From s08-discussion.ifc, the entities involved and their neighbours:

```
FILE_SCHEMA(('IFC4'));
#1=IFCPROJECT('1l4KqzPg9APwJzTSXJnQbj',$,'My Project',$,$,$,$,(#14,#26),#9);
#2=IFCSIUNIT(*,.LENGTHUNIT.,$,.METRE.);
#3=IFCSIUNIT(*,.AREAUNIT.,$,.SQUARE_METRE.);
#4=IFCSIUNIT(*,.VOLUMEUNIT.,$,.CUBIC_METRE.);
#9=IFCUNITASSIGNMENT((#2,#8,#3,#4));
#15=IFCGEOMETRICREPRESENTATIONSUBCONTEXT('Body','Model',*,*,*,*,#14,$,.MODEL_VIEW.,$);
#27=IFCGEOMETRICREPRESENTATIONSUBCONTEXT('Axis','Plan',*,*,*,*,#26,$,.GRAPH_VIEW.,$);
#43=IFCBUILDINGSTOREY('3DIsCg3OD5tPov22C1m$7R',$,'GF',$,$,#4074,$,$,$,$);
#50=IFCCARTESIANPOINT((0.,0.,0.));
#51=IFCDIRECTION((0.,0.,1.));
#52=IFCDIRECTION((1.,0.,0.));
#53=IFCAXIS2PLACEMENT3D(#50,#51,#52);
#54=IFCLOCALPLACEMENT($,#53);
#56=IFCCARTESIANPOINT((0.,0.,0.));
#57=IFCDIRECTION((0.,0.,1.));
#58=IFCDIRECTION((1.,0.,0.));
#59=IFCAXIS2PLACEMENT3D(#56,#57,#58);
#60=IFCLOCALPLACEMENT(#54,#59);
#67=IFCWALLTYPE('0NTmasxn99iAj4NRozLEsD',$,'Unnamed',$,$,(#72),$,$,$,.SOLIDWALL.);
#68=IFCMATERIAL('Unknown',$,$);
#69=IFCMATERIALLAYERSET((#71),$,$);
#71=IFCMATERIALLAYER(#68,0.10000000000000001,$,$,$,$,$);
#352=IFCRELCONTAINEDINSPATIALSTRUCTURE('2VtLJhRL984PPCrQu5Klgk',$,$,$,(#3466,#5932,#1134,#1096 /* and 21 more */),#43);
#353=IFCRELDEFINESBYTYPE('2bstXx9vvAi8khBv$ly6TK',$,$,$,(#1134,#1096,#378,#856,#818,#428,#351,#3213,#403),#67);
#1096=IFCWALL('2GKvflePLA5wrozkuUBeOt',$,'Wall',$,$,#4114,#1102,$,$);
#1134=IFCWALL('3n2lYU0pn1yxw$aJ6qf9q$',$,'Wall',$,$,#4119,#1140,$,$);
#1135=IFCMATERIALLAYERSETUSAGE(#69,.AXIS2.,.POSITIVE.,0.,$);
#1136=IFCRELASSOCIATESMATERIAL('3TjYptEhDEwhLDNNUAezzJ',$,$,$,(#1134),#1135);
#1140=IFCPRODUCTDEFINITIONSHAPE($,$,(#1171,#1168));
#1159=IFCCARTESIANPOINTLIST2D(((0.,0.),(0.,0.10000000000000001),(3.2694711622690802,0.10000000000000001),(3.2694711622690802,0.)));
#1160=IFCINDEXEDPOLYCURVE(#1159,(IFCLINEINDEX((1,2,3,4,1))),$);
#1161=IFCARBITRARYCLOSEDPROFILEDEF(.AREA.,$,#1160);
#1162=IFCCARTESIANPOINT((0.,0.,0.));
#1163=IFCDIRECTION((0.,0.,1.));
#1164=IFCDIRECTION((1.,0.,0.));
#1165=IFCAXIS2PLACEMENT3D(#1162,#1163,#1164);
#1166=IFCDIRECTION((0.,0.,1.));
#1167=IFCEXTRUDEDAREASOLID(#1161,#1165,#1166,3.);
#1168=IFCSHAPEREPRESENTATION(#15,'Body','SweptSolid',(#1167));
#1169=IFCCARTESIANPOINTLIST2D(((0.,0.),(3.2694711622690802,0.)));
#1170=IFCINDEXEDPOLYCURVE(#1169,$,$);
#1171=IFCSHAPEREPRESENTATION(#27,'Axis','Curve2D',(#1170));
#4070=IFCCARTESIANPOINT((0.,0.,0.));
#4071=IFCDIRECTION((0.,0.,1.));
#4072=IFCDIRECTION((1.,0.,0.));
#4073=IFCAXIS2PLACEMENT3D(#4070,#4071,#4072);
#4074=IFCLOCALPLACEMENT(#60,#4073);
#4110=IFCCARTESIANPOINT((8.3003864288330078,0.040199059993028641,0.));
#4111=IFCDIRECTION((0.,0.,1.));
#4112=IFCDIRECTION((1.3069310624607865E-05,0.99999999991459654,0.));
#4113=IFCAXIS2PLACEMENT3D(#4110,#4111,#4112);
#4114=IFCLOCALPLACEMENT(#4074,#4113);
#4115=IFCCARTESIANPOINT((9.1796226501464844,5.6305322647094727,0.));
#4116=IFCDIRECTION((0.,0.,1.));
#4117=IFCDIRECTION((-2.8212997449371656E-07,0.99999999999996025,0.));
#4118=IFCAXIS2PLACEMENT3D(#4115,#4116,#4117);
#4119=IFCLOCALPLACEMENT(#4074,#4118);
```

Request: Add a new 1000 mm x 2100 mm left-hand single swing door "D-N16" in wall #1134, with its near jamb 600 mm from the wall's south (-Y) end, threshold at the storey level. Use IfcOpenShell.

```python
import numpy as np
import ifcopenshell
import ifcopenshell.api.feature
import ifcopenshell.api.geometry
import ifcopenshell.api.root
import ifcopenshell.api.spatial
import ifcopenshell.geom
import ifcopenshell.util.element
import ifcopenshell.util.placement
import ifcopenshell.util.representation
import ifcopenshell.util.shape
import ifcopenshell.util.unit

model = ifcopenshell.open("s08-discussion.ifc")
unit_scale = ifcopenshell.util.unit.calculate_unit_scale(model)
settings = ifcopenshell.geom.settings()


def volume(element):
    """Net volume in cubic metres, openings subtracted."""
    shape = ifcopenshell.geom.create_shape(settings, element)
    return ifcopenshell.util.shape.get_volume(shape.geometry)


wall = model.by_guid("3n2lYU0pn1yxw$aJ6qf9q$")
storey = ifcopenshell.util.element.get_container(wall, ifc_class="IfcBuildingStorey")
context = ifcopenshell.util.representation.get_context(model, "Model", "Body", "MODEL_VIEW")
before = volume(wall)

width, height, from_end, sill = 1, 2.1, 0.6, 0.0  # metres

# The wall runs along its own X axis, and the end named is its -X end.
wall_shape = ifcopenshell.geom.create_shape(settings, wall)
x, y, z = ifcopenshell.util.shape.get_vertices(wall_shape.geometry).T
start = x.min() + from_end
face, thickness = float(y.min()), float(y.max() - y.min())
wall_matrix = ifcopenshell.util.placement.get_local_placement(wall.ObjectPlacement)
level = ifcopenshell.util.placement.get_local_placement(storey.ObjectPlacement)[2, 3]


def in_wall(x, y):
    """Placement at x, y metres in the wall's axes, at sill height."""
    matrix = wall_matrix.copy()
    matrix[:, 3] = wall_matrix @ np.array([x / unit_scale, y / unit_scale, 0.0, 1.0])
    matrix[2, 3] = level + sill / unit_scale
    return matrix


# Opening: a box that overshoots both wall faces by 50 mm.
opening = ifcopenshell.api.root.create_entity(model, ifc_class="IfcOpeningElement", predefined_type="OPENING")
box = ifcopenshell.api.geometry.add_wall_representation(
    model, context=context, length=width, height=height, thickness=thickness + 0.1
)
ifcopenshell.api.geometry.assign_representation(model, product=opening, representation=box)
ifcopenshell.api.geometry.edit_object_placement(model, product=opening, matrix=in_wall(start, face - 0.05), is_si=False)
ifcopenshell.api.feature.add_feature(model, feature=opening, element=wall)

door = ifcopenshell.api.root.create_entity(model, ifc_class="IfcDoor", name="D-N16", predefined_type="DOOR")
door.OverallWidth, door.OverallHeight = width / unit_scale, height / unit_scale
door.OperationType = "SINGLE_SWING_LEFT"
body = ifcopenshell.api.geometry.add_door_representation(
    model,
    context=context,
    overall_width=door.OverallWidth,
    overall_height=door.OverallHeight,
    operation_type="SINGLE_SWING_LEFT",
    lining_properties={"LiningDepth": thickness / unit_scale, "ThresholdDepth": thickness / unit_scale},
)
ifcopenshell.api.geometry.assign_representation(model, product=door, representation=body)
ifcopenshell.api.spatial.assign_container(model, products=[door], relating_structure=storey)
ifcopenshell.api.feature.add_filling(model, opening=opening, element=door)

# The lining spans the wall, so the door starts at the wall face.
ifcopenshell.api.geometry.edit_object_placement(model, product=door, matrix=in_wall(start, face), is_si=False)

after = volume(wall)

print(f"wall volume {before:.3f} -> {after:.3f} m3")

model.write("s08-discussion_updated.ifc")
```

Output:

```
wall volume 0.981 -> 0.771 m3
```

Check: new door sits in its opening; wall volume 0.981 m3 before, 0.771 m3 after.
